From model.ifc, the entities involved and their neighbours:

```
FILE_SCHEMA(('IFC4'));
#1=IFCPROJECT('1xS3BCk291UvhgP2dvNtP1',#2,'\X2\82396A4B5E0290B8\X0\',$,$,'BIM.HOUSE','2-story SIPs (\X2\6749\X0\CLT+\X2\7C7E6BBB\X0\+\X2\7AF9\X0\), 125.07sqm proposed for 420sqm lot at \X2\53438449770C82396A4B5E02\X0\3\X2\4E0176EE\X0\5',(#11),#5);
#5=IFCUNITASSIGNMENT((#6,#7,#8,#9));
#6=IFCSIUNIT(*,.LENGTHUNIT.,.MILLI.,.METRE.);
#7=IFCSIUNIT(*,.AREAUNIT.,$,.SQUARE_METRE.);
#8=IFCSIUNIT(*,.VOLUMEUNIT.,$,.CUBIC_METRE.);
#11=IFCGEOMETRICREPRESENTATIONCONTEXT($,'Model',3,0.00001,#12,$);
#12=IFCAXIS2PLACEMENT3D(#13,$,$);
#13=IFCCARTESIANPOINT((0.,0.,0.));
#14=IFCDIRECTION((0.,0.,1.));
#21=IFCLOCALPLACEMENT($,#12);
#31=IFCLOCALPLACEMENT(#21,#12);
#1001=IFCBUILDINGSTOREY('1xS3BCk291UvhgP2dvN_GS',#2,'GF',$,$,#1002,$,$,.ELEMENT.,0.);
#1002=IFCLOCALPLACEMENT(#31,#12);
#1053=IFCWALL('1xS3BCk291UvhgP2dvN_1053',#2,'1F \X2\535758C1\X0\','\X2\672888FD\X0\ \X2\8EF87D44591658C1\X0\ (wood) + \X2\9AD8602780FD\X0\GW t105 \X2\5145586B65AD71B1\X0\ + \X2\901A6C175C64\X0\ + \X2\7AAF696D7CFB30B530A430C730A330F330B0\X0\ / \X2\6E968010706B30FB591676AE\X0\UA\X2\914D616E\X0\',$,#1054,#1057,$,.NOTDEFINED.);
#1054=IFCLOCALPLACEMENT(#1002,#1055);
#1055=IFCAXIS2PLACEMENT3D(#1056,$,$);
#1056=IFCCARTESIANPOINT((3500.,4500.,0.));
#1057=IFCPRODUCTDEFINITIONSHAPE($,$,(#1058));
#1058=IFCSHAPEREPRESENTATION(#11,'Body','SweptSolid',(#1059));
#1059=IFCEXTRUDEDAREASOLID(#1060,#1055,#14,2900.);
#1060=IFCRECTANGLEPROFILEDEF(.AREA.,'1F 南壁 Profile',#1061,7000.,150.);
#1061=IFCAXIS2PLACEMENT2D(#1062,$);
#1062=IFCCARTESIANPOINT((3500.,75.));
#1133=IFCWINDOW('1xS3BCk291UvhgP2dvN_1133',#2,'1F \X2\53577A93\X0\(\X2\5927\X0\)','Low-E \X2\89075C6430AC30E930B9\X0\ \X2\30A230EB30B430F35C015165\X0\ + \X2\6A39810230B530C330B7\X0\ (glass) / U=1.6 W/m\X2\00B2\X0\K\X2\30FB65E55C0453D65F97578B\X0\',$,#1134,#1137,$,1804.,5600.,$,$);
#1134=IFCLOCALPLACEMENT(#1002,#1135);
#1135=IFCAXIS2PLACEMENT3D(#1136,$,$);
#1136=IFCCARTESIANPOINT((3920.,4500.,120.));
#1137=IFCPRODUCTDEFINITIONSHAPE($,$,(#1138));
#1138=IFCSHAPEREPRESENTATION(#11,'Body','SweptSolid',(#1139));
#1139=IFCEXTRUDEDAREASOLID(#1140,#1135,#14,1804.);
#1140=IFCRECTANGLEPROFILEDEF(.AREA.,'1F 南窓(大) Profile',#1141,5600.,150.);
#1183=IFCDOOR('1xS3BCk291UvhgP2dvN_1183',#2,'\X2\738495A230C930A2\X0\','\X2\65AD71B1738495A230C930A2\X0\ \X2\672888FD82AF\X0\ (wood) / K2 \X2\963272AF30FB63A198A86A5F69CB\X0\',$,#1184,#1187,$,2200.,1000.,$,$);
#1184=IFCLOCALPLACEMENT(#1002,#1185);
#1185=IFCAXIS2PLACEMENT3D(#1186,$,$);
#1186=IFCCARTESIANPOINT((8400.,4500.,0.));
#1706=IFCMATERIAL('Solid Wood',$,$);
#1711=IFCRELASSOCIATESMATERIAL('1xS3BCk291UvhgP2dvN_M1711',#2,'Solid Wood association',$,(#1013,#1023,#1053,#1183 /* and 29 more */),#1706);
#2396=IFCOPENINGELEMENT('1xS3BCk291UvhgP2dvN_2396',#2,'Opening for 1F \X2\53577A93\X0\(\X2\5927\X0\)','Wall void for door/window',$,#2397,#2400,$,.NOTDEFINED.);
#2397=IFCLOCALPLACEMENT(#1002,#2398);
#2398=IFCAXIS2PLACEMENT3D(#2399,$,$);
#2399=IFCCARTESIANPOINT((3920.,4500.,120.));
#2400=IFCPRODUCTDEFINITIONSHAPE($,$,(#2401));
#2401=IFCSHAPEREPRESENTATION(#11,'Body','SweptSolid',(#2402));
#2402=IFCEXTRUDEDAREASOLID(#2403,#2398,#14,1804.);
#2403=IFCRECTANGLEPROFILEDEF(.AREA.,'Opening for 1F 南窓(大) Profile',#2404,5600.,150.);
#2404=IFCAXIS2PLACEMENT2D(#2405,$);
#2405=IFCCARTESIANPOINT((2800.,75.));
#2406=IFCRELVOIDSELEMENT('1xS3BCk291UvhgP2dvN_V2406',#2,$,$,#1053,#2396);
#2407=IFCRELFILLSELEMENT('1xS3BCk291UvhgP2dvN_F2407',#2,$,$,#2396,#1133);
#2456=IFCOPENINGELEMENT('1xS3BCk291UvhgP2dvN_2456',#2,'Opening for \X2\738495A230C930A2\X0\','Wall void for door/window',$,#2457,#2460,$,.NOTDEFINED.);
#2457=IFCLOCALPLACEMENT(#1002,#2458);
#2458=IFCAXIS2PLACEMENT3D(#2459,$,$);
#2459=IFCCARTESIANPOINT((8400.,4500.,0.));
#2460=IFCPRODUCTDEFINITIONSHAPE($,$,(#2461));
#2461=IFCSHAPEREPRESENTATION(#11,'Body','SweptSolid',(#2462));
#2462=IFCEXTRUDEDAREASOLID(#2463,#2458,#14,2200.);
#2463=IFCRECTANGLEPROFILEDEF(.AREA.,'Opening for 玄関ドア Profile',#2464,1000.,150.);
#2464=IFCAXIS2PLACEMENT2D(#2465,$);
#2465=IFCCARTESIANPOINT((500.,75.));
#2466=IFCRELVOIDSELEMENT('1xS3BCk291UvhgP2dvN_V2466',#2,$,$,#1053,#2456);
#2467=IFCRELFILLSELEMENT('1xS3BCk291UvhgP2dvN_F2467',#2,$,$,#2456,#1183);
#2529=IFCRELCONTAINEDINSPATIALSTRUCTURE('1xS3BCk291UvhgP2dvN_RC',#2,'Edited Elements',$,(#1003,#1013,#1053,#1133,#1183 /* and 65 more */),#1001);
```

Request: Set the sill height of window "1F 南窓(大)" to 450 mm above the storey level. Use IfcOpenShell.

```python
import numpy as np
import ifcopenshell
import ifcopenshell.api.geometry
import ifcopenshell.geom
import ifcopenshell.util.element
import ifcopenshell.util.placement
import ifcopenshell.util.shape
import ifcopenshell.util.unit

model = ifcopenshell.open("model.ifc")
unit_scale = ifcopenshell.util.unit.calculate_unit_scale(model)

window = model.by_guid("1xS3BCk291UvhgP2dvN_1133")
opening = window.FillsVoids[0].RelatingOpeningElement
storey = ifcopenshell.util.element.get_container(window, ifc_class="IfcBuildingStorey")
level = ifcopenshell.util.placement.get_local_placement(storey.ObjectPlacement)[2, 3]

# The opening's origin need not be at the sill, so measure its lowest point.
shape = ifcopenshell.geom.create_shape(ifcopenshell.geom.settings(), opening)
bottom = ifcopenshell.util.shape.get_shape_bottom_elevation(shape, shape.geometry) / unit_scale
dz = level + 0.45 / unit_scale - bottom

shift = np.array([0.0, 0.0, dz])
# The window is not placed relative to its opening, so move both.
for product in (opening, window):
    matrix = ifcopenshell.util.placement.get_local_placement(product.ObjectPlacement)
    matrix[:3, 3] += shift
    ifcopenshell.api.geometry.edit_object_placement(model, product=product, matrix=matrix, is_si=False)

print(f"moved by {dz * unit_scale:+.3f} m")

model.write("model_rev.ifc")
```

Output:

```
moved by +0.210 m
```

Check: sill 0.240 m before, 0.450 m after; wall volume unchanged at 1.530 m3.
